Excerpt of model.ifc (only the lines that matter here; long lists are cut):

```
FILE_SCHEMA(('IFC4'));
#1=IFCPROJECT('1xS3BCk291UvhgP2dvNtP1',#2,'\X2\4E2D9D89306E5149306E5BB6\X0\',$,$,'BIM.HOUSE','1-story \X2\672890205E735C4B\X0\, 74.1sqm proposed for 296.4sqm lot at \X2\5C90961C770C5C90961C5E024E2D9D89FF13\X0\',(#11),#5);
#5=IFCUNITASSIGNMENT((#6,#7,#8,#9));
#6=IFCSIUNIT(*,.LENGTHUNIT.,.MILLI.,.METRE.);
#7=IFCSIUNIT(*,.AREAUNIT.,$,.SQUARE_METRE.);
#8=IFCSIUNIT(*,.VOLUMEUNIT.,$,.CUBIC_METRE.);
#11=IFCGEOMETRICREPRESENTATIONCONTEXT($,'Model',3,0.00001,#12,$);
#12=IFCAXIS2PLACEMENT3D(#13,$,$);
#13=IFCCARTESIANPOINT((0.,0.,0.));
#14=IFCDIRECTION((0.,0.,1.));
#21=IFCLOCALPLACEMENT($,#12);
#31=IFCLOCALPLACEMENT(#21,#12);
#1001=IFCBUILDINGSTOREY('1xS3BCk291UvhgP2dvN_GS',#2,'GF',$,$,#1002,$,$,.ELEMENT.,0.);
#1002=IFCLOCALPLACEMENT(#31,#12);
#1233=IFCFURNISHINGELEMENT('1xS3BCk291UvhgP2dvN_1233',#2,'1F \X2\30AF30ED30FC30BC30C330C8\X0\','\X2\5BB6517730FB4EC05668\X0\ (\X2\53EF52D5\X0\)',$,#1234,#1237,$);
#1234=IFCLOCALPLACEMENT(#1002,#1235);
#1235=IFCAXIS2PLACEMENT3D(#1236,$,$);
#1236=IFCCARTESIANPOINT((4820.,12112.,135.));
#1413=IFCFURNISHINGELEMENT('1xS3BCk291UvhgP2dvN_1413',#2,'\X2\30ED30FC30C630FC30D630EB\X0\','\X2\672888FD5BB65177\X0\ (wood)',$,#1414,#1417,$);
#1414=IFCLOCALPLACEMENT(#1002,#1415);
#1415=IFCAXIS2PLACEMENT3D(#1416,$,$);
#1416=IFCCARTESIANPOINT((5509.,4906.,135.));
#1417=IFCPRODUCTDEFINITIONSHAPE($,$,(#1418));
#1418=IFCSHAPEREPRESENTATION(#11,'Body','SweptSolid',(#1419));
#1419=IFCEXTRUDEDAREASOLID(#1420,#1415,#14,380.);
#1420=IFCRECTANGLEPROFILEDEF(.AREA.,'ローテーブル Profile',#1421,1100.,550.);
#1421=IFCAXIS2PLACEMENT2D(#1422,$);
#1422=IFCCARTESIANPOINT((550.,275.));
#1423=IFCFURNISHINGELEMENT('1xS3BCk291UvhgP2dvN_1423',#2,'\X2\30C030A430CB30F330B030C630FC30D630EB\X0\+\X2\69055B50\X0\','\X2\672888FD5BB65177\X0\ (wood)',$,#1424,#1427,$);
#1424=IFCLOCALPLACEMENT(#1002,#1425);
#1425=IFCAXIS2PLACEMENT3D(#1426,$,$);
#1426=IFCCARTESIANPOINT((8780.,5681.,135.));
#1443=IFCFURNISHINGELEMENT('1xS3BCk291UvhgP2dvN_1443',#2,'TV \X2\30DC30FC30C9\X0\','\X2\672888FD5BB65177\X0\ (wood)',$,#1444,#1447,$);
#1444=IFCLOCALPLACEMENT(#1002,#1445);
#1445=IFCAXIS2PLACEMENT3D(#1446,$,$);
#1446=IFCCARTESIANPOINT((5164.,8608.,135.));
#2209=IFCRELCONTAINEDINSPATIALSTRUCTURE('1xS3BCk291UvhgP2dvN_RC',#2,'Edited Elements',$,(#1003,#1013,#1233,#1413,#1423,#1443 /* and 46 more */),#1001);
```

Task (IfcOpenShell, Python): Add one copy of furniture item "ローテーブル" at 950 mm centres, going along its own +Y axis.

```python
import ifcopenshell
import ifcopenshell.api.geometry
import ifcopenshell.api.root
import ifcopenshell.util.element
import ifcopenshell.util.placement
import ifcopenshell.util.unit

model = ifcopenshell.open("model.ifc")
unit_scale = ifcopenshell.util.unit.calculate_unit_scale(model)


def reuse_history(source, copy):
    """copy_class also copies each property set's owner history, people and application; keep the originals."""
    for rel in copy.IsDefinedBy:
        if rel.is_a("IfcRelDefinesByProperties") and (history := rel.RelatingPropertyDefinition.OwnerHistory):
            rel.RelatingPropertyDefinition.OwnerHistory = source.OwnerHistory
            ifcopenshell.util.element.remove_deep2(model, history)


source = model.by_guid("1xS3BCk291UvhgP2dvN_1413")
base = ifcopenshell.util.placement.get_local_placement(source.ObjectPlacement)
step = base[:3, 1] * 0.95 / unit_scale

for i in range(1, 2):
    copy = ifcopenshell.api.root.copy_class(model, product=source)
    copy.Representation = ifcopenshell.util.element.copy_deep(
        model, source.Representation, exclude=["IfcGeometricRepresentationContext", "IfcRepresentationMap"]
    )
    reuse_history(source, copy)
    matrix = base.copy()
    matrix[:3, 3] += i * step
    print("added at", matrix[:3, 3].round(3) + 0.0)
    ifcopenshell.api.geometry.edit_object_placement(model, product=copy, matrix=matrix, is_si=False)

model.write("model_edited.ifc")
```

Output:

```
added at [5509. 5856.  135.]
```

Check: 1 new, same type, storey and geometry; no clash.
